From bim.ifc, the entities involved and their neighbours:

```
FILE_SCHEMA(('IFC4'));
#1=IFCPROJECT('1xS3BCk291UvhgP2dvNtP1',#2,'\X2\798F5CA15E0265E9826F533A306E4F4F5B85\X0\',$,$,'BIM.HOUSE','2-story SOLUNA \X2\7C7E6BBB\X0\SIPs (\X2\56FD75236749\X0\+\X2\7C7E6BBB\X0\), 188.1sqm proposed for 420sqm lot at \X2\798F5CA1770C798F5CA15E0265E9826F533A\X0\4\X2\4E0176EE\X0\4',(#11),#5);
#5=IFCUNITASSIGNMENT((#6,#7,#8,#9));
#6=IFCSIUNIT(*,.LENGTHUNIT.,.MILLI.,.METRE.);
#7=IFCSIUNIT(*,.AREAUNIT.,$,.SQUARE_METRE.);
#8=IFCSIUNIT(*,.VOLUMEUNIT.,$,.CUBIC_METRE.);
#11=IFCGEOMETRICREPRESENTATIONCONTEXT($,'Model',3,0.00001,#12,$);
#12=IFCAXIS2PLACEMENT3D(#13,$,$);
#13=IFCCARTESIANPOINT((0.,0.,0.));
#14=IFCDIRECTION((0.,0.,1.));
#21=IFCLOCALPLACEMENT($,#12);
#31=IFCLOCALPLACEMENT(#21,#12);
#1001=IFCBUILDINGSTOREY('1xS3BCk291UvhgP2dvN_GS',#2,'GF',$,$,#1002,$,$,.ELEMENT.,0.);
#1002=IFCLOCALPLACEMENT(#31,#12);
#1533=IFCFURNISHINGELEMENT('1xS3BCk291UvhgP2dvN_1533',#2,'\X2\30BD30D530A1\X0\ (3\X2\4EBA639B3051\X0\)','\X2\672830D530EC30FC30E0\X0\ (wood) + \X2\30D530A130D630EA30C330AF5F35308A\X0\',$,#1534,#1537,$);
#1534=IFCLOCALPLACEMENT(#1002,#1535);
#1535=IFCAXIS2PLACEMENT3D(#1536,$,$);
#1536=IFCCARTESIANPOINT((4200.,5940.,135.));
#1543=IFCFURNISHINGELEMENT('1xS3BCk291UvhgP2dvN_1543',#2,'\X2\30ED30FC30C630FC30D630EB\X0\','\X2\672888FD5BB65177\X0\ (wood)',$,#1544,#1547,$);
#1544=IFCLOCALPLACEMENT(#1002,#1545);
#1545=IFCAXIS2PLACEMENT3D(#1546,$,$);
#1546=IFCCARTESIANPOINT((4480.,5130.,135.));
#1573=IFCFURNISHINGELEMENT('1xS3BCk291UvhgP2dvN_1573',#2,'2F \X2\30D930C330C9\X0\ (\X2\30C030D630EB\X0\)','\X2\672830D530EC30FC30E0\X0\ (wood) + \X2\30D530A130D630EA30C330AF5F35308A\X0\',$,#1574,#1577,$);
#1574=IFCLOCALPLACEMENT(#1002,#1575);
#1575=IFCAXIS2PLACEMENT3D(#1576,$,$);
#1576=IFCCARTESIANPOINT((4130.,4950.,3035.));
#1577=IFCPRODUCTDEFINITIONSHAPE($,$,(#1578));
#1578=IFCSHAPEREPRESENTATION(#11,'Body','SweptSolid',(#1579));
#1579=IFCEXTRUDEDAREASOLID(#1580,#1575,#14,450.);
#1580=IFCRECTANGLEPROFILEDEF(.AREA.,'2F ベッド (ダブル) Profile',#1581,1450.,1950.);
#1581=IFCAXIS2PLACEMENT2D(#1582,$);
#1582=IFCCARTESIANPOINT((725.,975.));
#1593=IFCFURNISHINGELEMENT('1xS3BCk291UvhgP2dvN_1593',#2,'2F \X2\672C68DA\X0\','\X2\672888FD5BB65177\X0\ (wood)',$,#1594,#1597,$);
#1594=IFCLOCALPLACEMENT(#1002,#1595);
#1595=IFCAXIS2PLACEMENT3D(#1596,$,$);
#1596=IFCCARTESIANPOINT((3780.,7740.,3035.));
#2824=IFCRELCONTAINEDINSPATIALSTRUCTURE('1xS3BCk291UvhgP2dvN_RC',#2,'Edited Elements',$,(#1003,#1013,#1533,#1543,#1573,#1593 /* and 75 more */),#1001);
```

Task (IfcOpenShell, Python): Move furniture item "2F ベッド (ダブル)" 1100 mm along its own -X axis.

```python
import ifcopenshell
import ifcopenshell.api.geometry
import ifcopenshell.util.placement

model = ifcopenshell.open("bim.ifc")

item = model.by_id(1573)
matrix = ifcopenshell.util.placement.get_local_placement(item.ObjectPlacement)
matrix[:3, 3] -= matrix[:3, 0] * 1100.0
ifcopenshell.api.geometry.edit_object_placement(model, product=item, matrix=matrix, is_si=False)

print(ifcopenshell.util.placement.get_local_placement(item.ObjectPlacement).round(3) + 0.0)

model.write("bim-out.ifc")
```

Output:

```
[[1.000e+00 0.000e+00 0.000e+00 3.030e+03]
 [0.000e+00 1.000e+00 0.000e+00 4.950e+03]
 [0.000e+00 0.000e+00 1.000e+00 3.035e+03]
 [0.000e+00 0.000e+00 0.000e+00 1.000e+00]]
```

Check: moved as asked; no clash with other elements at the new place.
